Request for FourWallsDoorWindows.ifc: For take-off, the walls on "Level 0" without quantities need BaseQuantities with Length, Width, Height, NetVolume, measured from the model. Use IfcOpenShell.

First a look at what the model holds.

```python
import ifcopenshell
import ifcopenshell.util.element
import ifcopenshell.util.unit

model = ifcopenshell.open("FourWallsDoorWindows.ifc")
print(model.schema)
for unit_type in ("LENGTHUNIT", "AREAUNIT", "VOLUMEUNIT"):
    print(unit_type, ifcopenshell.util.unit.calculate_unit_scale(model, unit_type))
storey = next(s for s in model.by_type("IfcBuildingStorey") if s.Name == "Level 0")
walls = [e for e in ifcopenshell.util.element.get_decomposition(storey) if e.is_a("IfcWall")]
for e in sorted(walls, key=lambda e: e.id()):
    print(e.id(), e.is_a(), e.Name, list(ifcopenshell.util.element.get_psets(e, qtos_only=True)), sep=" | ")
```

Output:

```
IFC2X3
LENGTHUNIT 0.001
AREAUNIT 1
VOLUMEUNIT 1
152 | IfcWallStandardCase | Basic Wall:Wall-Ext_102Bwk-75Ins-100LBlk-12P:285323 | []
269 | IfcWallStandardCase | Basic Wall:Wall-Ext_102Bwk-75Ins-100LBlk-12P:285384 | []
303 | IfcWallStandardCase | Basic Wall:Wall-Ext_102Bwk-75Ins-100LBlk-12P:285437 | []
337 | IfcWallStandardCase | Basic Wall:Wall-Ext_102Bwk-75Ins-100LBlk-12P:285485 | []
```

```python
import ifcopenshell
import ifcopenshell.api.pset
import ifcopenshell.geom
import ifcopenshell.util.element
import ifcopenshell.util.shape
import ifcopenshell.util.unit

model = ifcopenshell.open("FourWallsDoorWindows.ifc")
unit_scale = ifcopenshell.util.unit.calculate_unit_scale(model)
volume_scale = ifcopenshell.util.unit.calculate_unit_scale(model, "VOLUMEUNIT")
settings = ifcopenshell.geom.settings()

storey = next(s for s in model.by_type("IfcBuildingStorey") if s.Name == "Level 0")
walls = [e for e in ifcopenshell.util.element.get_decomposition(storey) if e.is_a("IfcWall")]

for e in sorted(walls, key=lambda e: e.id()):
    if ifcopenshell.util.element.get_psets(e, qtos_only=True, should_inherit=False):
        continue
    # Geometry comes back in metres, in the element's own axes.
    shape = ifcopenshell.geom.create_shape(settings, e)
    values = {
        "Length": ifcopenshell.util.shape.get_x(shape.geometry) / unit_scale,
        "Width": ifcopenshell.util.shape.get_y(shape.geometry) / unit_scale,
        "Height": ifcopenshell.util.shape.get_z(shape.geometry) / unit_scale,
        "NetVolume": ifcopenshell.util.shape.get_volume(shape.geometry) / volume_scale,
    }
    qto = ifcopenshell.api.pset.add_qto(model, product=e, name="BaseQuantities")
    ifcopenshell.api.pset.edit_qto(model, qto=qto, properties=values)
    print(e.id(), {k: round(v, 3) for k, v in values.items()})

model.write("FourWallsDoorWindows_v2.ifc")
```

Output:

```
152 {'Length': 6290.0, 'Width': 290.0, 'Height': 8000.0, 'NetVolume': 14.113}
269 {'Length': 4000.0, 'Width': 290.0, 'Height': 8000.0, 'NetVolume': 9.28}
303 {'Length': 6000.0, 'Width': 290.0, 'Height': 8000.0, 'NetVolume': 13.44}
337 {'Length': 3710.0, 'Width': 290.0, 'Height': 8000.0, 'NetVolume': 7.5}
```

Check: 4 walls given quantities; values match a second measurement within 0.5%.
